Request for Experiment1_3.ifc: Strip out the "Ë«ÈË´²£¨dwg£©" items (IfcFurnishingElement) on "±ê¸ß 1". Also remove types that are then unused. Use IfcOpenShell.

First a look at what the model holds.

```python
import ifcopenshell
import ifcopenshell.util.element

model = ifcopenshell.open("Experiment1_3.ifc")
print(model.schema)
storey = next(s for s in model.by_type("IfcBuildingStorey") if s.Name == "±ê¸ß 1")
furniture = [e for e in ifcopenshell.util.element.get_decomposition(storey) if e.is_a("IfcFurnishingElement")]
seen = {}
for e in furniture:
    element_type = ifcopenshell.util.element.get_type(e)
    name = element_type.Name if element_type not in (None, e) else None
    seen[name] = seen.get(name, 0) + 1
for name, count in sorted(seen.items(), key=str):
    print(count, "x", name)
```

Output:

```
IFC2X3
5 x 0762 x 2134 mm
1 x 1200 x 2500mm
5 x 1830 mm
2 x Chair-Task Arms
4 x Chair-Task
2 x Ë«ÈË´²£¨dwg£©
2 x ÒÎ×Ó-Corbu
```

```python
import ifcopenshell
import ifcopenshell.api.root
import ifcopenshell.util.element

model = ifcopenshell.open("Experiment1_3.ifc")

storey = next(s for s in model.by_type("IfcBuildingStorey") if s.Name == "±ê¸ß 1")
furniture = [e for e in ifcopenshell.util.element.get_decomposition(storey) if e.is_a("IfcFurnishingElement")]
targets = [e for e in furniture if (t := ifcopenshell.util.element.get_type(e)) not in (None, e) and t.Name == "Ë«ÈË´²£¨dwg£©"]
types = {ifcopenshell.util.element.get_type(e) for e in targets} - {None, *targets}

for e in targets:
    ifcopenshell.api.root.remove_product(model, product=e)
print(len(targets), "removed")

unused = [t for t in types if not ifcopenshell.util.element.get_types(t)]
for t in unused:
    ifcopenshell.api.root.remove_product(model, product=t)
print(len(unused), "unused types removed")

model.write("Experiment1_3_edited.ifc")
```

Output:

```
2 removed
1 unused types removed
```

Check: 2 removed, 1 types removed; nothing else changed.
